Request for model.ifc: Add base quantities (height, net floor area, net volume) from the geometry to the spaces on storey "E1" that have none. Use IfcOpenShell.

First a look at what the model holds.

```python
import ifcopenshell
import ifcopenshell.util.element
import ifcopenshell.util.unit

model = ifcopenshell.open("model.ifc")
print(model.schema)
for unit_type in ("LENGTHUNIT", "AREAUNIT", "VOLUMEUNIT"):
    print(unit_type, ifcopenshell.util.unit.calculate_unit_scale(model, unit_type))
storey = next(s for s in model.by_type("IfcBuildingStorey") if s.Name == "E1")
spaces = [e for e in ifcopenshell.util.element.get_decomposition(storey) if e.is_a("IfcSpace")]
for e in sorted(spaces, key=lambda e: e.id()):
    print(e.id(), e.is_a(), e.Name, list(ifcopenshell.util.element.get_psets(e, qtos_only=True)), sep=" | ")
```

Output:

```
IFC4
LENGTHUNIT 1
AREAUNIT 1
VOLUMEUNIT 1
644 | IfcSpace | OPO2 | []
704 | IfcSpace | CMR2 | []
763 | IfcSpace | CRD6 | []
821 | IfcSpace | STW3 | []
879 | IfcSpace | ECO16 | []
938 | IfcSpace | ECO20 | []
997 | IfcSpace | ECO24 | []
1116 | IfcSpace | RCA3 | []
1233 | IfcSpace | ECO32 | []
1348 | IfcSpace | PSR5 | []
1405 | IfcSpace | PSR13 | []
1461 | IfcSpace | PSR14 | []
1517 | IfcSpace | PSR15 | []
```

```python
import ifcopenshell
import ifcopenshell.api.pset
import ifcopenshell.geom
import ifcopenshell.util.element
import ifcopenshell.util.shape
import ifcopenshell.util.unit

model = ifcopenshell.open("model.ifc")
unit_scale = ifcopenshell.util.unit.calculate_unit_scale(model)
area_scale = ifcopenshell.util.unit.calculate_unit_scale(model, "AREAUNIT")
volume_scale = ifcopenshell.util.unit.calculate_unit_scale(model, "VOLUMEUNIT")
settings = ifcopenshell.geom.settings()

storey = next(s for s in model.by_type("IfcBuildingStorey") if s.Name == "E1")
spaces = [e for e in ifcopenshell.util.element.get_decomposition(storey) if e.is_a("IfcSpace")]

for e in sorted(spaces, key=lambda e: e.id()):
    if ifcopenshell.util.element.get_psets(e, qtos_only=True, should_inherit=False):
        continue
    # Geometry comes back in metres, in the element's own axes.
    shape = ifcopenshell.geom.create_shape(settings, e)
    values = {
        "Height": ifcopenshell.util.shape.get_z(shape.geometry) / unit_scale,
        "NetFloorArea": ifcopenshell.util.shape.get_footprint_area(shape.geometry) / area_scale,
        "NetVolume": ifcopenshell.util.shape.get_volume(shape.geometry) / volume_scale,
    }
    qto = ifcopenshell.api.pset.add_qto(model, product=e, name="Qto_SpaceBaseQuantities")
    ifcopenshell.api.pset.edit_qto(model, qto=qto, properties=values)
    print(e.id(), {k: round(v, 3) for k, v in values.items()})

model.write("model_edited.ifc")
```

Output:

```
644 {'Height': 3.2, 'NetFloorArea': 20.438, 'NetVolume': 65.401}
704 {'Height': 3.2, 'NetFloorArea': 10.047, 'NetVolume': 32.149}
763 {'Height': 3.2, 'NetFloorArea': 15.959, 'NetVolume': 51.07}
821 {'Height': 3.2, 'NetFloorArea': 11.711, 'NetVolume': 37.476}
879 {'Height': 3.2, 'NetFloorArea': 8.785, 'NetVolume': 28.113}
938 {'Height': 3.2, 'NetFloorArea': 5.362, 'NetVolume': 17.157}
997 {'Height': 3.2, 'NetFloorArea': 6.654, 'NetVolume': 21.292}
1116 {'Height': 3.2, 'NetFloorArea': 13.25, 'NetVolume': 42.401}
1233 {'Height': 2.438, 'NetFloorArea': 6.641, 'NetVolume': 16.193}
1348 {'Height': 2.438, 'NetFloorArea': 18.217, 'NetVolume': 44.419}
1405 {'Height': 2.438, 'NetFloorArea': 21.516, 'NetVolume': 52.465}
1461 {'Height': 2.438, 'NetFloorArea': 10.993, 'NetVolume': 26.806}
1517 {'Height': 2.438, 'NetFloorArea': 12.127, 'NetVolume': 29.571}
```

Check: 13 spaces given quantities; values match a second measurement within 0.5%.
